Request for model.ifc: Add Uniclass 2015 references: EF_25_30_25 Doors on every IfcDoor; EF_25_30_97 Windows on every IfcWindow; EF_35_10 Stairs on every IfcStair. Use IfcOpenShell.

First a look at what the model holds.

```python
import ifcopenshell

model = ifcopenshell.open("model.ifc")
print(model.schema)
print("classifications:", [c.Name for c in model.by_type("IfcClassification")])
for ifc_class in ("IfcDoor", "IfcRoof", "IfcStair", "IfcWall", "IfcWindow"):
    print(ifc_class, len(model.by_type(ifc_class)))
```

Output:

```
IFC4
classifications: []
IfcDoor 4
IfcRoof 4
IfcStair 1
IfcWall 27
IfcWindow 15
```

```python
import ifcopenshell
import ifcopenshell.api.classification

model = ifcopenshell.open("model.ifc")

system = ifcopenshell.api.classification.add_classification(model, classification="Uniclass 2015")

codes = {
    "IfcDoor": ("EF_25_30_25", "Doors"),
    "IfcWindow": ("EF_25_30_97", "Windows"),
    "IfcStair": ("EF_35_10", "Stairs"),
}
for ifc_class, (code, name) in codes.items():
    products = model.by_type(ifc_class)
    ifcopenshell.api.classification.add_reference(
        model, products=products, classification=system, identification=code, name=name
    )
    print(code, len(products))

model.write("model-out.ifc")
```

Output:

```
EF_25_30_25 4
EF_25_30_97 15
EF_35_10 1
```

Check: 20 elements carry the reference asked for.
